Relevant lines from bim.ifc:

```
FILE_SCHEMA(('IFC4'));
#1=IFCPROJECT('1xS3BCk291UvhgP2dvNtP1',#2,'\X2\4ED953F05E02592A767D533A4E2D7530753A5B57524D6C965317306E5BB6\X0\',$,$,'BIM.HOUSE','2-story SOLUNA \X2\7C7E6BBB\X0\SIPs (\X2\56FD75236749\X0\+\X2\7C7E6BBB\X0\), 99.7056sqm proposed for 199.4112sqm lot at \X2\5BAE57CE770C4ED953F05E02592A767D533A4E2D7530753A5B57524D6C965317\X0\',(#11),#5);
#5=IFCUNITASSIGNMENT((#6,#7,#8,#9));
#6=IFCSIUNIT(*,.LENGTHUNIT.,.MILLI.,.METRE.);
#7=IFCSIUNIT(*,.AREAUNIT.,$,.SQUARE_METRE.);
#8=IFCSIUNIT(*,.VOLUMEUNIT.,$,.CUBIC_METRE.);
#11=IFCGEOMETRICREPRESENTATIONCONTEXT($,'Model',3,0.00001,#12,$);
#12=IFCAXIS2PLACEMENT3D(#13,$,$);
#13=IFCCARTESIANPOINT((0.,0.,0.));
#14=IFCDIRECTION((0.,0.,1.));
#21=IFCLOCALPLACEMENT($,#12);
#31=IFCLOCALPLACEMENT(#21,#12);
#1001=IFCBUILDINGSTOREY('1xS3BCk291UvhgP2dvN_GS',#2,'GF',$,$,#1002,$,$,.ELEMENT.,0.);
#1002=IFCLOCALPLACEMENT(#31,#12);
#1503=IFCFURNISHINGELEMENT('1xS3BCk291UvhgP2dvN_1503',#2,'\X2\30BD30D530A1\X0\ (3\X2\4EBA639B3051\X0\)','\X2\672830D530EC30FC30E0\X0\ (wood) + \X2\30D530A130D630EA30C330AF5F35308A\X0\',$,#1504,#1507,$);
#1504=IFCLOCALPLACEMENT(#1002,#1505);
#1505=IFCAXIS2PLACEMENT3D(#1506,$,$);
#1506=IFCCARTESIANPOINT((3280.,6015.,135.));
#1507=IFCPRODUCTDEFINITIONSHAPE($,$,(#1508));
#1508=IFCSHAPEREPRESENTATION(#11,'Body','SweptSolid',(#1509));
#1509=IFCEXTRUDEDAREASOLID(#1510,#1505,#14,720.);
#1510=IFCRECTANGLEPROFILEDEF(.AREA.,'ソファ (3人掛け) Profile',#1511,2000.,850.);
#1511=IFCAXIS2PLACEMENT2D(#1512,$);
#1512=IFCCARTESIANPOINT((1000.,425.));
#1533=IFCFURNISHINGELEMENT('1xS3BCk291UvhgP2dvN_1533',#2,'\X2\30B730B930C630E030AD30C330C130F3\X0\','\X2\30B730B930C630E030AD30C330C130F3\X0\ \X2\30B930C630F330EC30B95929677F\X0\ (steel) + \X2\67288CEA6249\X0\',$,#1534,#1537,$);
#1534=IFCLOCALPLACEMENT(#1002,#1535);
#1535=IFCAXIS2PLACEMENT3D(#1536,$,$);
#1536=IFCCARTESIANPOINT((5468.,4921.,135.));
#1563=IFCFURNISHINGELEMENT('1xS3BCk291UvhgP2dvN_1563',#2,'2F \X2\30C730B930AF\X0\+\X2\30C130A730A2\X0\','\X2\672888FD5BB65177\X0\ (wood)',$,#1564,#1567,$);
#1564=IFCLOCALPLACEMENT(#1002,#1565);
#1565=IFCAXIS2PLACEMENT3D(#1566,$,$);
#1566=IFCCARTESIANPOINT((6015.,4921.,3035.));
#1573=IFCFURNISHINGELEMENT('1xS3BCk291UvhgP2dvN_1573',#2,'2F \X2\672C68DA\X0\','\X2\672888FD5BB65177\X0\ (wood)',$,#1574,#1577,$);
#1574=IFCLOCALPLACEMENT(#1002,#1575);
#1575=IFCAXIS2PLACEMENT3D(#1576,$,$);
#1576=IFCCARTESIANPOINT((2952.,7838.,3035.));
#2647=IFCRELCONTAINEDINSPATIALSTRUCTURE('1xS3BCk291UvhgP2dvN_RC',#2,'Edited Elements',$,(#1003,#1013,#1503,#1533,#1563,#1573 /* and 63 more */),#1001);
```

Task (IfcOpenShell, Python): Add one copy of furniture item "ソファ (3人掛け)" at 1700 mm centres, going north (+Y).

```python
import numpy as np
import ifcopenshell
import ifcopenshell.api.geometry
import ifcopenshell.api.root
import ifcopenshell.util.element
import ifcopenshell.util.placement

model = ifcopenshell.open("bim.ifc")


def reuse_history(source, copy):
    """copy_class also copies each property set's owner history, people and application; keep the originals."""
    for rel in copy.IsDefinedBy:
        if rel.is_a("IfcRelDefinesByProperties") and (history := rel.RelatingPropertyDefinition.OwnerHistory):
            rel.RelatingPropertyDefinition.OwnerHistory = source.OwnerHistory
            ifcopenshell.util.element.remove_deep2(model, history)


source = model.by_id(1503)
base = ifcopenshell.util.placement.get_local_placement(source.ObjectPlacement)
step = np.array([0.0, 1.0, 0.0]) * 1700.0

for i in range(1, 2):
    copy = ifcopenshell.api.root.copy_class(model, product=source)
    copy.Representation = ifcopenshell.util.element.copy_deep(
        model, source.Representation, exclude=["IfcGeometricRepresentationContext", "IfcRepresentationMap"]
    )
    reuse_history(source, copy)
    matrix = base.copy()
    matrix[:3, 3] += i * step
    print("added at", matrix[:3, 3].round(3) + 0.0)
    ifcopenshell.api.geometry.edit_object_placement(model, product=copy, matrix=matrix, is_si=False)

model.write("bim-out.ifc")
```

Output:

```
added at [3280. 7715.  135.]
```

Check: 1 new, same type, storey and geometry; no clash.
